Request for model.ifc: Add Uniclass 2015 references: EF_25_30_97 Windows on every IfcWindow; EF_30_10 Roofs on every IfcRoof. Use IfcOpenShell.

First a look at what the model holds.

```python
import ifcopenshell

model = ifcopenshell.open("model.ifc")
print(model.schema)
print("classifications:", [c.Name for c in model.by_type("IfcClassification")])
for ifc_class in ("IfcDoor", "IfcRoof", "IfcStair", "IfcWall", "IfcWindow"):
    print(ifc_class, len(model.by_type(ifc_class)))
```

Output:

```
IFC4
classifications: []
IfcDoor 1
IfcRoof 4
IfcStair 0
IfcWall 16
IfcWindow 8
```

```python
import ifcopenshell
import ifcopenshell.api.classification

model = ifcopenshell.open("model.ifc")

system = ifcopenshell.api.classification.add_classification(model, classification="Uniclass 2015")

codes = {
    "IfcWindow": ("EF_25_30_97", "Windows"),
    "IfcRoof": ("EF_30_10", "Roofs"),
}
for ifc_class, (code, name) in codes.items():
    products = model.by_type(ifc_class)
    ifcopenshell.api.classification.add_reference(
        model, products=products, classification=system, identification=code, name=name
    )
    print(code, len(products))

model.write("model_updated.ifc")
```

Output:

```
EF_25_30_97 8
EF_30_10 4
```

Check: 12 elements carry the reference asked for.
